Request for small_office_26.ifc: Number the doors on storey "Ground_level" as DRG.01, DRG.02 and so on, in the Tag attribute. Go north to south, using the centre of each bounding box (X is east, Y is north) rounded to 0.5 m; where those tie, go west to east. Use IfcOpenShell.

First a look at what the model holds.

```python
import ifcopenshell
import ifcopenshell.util.element
import ifcopenshell.util.placement

model = ifcopenshell.open("small_office_26.ifc")
print(model.schema)
storey = next(s for s in model.by_type("IfcBuildingStorey") if s.Name == "Ground_level")
doors = [e for e in ifcopenshell.util.element.get_decomposition(storey) if e.is_a("IfcDoor")]
for e in sorted(doors, key=lambda e: e.id()):
    origin = ifcopenshell.util.placement.get_local_placement(e.ObjectPlacement)[:3, 3]
    print(e.id(), e.Tag, e.Name, origin.round(2) + 0.0, sep=" | ")
```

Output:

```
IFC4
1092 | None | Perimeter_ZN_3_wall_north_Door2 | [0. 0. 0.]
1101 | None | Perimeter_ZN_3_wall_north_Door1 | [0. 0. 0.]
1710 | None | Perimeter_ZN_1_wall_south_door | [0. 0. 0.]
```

```python
import ifcopenshell
import ifcopenshell.geom
import ifcopenshell.util.element
import ifcopenshell.util.shape

model = ifcopenshell.open("small_office_26.ifc")
settings = ifcopenshell.geom.settings()
settings.set("use-world-coords", True)


def centre(element):
    shape = ifcopenshell.geom.create_shape(settings, element)
    return ifcopenshell.util.shape.get_bbox_centroid(shape.geometry)


storey = next(s for s in model.by_type("IfcBuildingStorey") if s.Name == "Ground_level")
doors = [e for e in ifcopenshell.util.element.get_decomposition(storey) if e.is_a("IfcDoor")]

# Insertion points can sit at a corner or the storey origin, so sort by the geometry (in metres).
centres = {e: centre(e) for e in doors}
doors.sort(key=lambda e: (-round(centres[e][1] / 0.5), centres[e][0]))

for i, e in enumerate(doors, start=1):
    number = f"DRG.{i:02d}"
    e.Tag = number
    print(e.id(), number)

model.write("small_office_26_edited.ifc")
```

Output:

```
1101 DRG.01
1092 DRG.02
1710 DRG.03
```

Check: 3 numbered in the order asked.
